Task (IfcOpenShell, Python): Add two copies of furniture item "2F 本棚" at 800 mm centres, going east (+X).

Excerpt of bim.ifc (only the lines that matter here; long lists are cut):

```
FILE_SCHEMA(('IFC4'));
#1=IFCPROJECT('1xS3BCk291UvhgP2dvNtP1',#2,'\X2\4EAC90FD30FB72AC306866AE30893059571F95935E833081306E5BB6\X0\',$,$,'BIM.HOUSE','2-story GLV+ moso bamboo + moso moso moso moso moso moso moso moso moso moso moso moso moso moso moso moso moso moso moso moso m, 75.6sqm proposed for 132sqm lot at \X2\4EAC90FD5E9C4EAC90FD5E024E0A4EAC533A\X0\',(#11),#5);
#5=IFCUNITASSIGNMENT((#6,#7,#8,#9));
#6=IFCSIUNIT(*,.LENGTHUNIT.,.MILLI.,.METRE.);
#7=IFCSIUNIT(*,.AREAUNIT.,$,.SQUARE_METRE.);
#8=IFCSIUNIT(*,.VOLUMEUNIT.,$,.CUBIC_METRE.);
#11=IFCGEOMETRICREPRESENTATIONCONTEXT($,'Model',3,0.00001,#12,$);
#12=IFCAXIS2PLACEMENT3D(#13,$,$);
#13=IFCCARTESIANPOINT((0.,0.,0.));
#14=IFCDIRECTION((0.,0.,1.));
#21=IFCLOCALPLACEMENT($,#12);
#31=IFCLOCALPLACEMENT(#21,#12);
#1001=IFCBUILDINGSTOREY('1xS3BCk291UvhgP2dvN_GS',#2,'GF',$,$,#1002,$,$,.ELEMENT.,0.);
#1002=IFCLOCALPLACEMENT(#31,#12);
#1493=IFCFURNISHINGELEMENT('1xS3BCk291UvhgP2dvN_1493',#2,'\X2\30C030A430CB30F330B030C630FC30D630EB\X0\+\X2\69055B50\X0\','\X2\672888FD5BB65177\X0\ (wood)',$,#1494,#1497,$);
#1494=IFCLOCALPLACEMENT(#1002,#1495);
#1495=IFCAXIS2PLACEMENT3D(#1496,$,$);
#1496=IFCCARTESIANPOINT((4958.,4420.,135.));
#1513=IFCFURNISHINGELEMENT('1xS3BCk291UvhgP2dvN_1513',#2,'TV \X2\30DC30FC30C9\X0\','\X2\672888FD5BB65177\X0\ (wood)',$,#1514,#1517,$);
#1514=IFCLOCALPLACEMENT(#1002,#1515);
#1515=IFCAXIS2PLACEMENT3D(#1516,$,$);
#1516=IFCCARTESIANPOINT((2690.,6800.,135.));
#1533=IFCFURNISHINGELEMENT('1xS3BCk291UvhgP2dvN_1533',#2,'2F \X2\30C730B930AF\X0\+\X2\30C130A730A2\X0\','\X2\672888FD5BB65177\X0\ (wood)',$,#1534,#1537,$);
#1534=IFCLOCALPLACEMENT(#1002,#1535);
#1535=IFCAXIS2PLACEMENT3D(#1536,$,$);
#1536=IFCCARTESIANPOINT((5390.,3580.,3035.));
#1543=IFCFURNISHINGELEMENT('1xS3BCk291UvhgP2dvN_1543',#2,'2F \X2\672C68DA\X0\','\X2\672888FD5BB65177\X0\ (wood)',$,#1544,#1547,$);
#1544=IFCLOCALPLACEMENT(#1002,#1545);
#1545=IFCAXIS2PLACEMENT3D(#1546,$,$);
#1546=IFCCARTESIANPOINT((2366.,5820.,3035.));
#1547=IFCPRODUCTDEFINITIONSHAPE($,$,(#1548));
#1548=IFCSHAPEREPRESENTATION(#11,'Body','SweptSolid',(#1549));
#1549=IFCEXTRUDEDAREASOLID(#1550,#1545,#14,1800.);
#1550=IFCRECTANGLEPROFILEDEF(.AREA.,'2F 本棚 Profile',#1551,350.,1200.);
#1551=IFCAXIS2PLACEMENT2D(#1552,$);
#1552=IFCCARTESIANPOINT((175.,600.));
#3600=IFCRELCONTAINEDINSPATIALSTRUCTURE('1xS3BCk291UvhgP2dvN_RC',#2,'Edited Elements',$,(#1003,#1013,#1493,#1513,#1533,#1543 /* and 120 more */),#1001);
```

```python
import numpy as np
import ifcopenshell
import ifcopenshell.api.geometry
import ifcopenshell.api.root
import ifcopenshell.util.element
import ifcopenshell.util.placement
import ifcopenshell.util.unit

model = ifcopenshell.open("bim.ifc")
unit_scale = ifcopenshell.util.unit.calculate_unit_scale(model)


def reuse_history(source, copy):
    """copy_class also copies each property set's owner history, people and application; keep the originals."""
    for rel in copy.IsDefinedBy:
        if rel.is_a("IfcRelDefinesByProperties") and (history := rel.RelatingPropertyDefinition.OwnerHistory):
            rel.RelatingPropertyDefinition.OwnerHistory = source.OwnerHistory
            ifcopenshell.util.element.remove_deep2(model, history)


source = model.by_guid("1xS3BCk291UvhgP2dvN_1543")
base = ifcopenshell.util.placement.get_local_placement(source.ObjectPlacement)
step = np.array([1.0, 0.0, 0.0]) * 0.8 / unit_scale

for i in range(1, 3):
    copy = ifcopenshell.api.root.copy_class(model, product=source)
    copy.Representation = ifcopenshell.util.element.copy_deep(
        model, source.Representation, exclude=["IfcGeometricRepresentationContext", "IfcRepresentationMap"]
    )
    reuse_history(source, copy)
    matrix = base.copy()
    matrix[:3, 3] += i * step
    print("added at", matrix[:3, 3].round(3) + 0.0)
    ifcopenshell.api.geometry.edit_object_placement(model, product=copy, matrix=matrix, is_si=False)

model.write("bim-out.ifc")
```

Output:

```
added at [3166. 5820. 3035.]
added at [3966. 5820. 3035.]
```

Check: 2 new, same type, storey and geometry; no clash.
